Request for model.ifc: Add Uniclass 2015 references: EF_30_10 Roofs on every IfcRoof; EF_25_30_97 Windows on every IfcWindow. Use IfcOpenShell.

First a look at what the model holds.

```python
import ifcopenshell

model = ifcopenshell.open("model.ifc")
print(model.schema)
print("classifications:", [c.Name for c in model.by_type("IfcClassification")])
for ifc_class in ("IfcDoor", "IfcRoof", "IfcStair", "IfcWall", "IfcWindow"):
    print(ifc_class, len(model.by_type(ifc_class)))
```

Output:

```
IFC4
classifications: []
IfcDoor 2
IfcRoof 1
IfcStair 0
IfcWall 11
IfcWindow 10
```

```python
import ifcopenshell
import ifcopenshell.api.classification

model = ifcopenshell.open("model.ifc")

system = ifcopenshell.api.classification.add_classification(model, classification="Uniclass 2015")

codes = {
    "IfcRoof": ("EF_30_10", "Roofs"),
    "IfcWindow": ("EF_25_30_97", "Windows"),
}
for ifc_class, (code, name) in codes.items():
    products = model.by_type(ifc_class)
    ifcopenshell.api.classification.add_reference(
        model, products=products, classification=system, identification=code, name=name
    )
    print(code, len(products))

model.write("model-out.ifc")
```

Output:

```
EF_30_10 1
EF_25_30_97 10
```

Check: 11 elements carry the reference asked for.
